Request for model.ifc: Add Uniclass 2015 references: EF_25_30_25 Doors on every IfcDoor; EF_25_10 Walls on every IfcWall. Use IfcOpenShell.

First a look at what the model holds.

```python
import ifcopenshell

model = ifcopenshell.open("model.ifc")
print(model.schema)
print("classifications:", [c.Name for c in model.by_type("IfcClassification")])
for ifc_class in ("IfcDoor", "IfcRoof", "IfcStair", "IfcWall", "IfcWindow"):
    print(ifc_class, len(model.by_type(ifc_class)))
```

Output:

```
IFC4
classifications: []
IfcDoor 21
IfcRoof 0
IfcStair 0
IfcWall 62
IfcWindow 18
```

```python
import ifcopenshell
import ifcopenshell.api.classification

model = ifcopenshell.open("model.ifc")

system = ifcopenshell.api.classification.add_classification(model, classification="Uniclass 2015")

codes = {
    "IfcDoor": ("EF_25_30_25", "Doors"),
    "IfcWall": ("EF_25_10", "Walls"),
}
for ifc_class, (code, name) in codes.items():
    products = model.by_type(ifc_class)
    ifcopenshell.api.classification.add_reference(
        model, products=products, classification=system, identification=code, name=name
    )
    print(code, len(products))

model.write("model-out.ifc")
```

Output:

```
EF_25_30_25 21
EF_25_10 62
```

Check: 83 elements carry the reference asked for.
